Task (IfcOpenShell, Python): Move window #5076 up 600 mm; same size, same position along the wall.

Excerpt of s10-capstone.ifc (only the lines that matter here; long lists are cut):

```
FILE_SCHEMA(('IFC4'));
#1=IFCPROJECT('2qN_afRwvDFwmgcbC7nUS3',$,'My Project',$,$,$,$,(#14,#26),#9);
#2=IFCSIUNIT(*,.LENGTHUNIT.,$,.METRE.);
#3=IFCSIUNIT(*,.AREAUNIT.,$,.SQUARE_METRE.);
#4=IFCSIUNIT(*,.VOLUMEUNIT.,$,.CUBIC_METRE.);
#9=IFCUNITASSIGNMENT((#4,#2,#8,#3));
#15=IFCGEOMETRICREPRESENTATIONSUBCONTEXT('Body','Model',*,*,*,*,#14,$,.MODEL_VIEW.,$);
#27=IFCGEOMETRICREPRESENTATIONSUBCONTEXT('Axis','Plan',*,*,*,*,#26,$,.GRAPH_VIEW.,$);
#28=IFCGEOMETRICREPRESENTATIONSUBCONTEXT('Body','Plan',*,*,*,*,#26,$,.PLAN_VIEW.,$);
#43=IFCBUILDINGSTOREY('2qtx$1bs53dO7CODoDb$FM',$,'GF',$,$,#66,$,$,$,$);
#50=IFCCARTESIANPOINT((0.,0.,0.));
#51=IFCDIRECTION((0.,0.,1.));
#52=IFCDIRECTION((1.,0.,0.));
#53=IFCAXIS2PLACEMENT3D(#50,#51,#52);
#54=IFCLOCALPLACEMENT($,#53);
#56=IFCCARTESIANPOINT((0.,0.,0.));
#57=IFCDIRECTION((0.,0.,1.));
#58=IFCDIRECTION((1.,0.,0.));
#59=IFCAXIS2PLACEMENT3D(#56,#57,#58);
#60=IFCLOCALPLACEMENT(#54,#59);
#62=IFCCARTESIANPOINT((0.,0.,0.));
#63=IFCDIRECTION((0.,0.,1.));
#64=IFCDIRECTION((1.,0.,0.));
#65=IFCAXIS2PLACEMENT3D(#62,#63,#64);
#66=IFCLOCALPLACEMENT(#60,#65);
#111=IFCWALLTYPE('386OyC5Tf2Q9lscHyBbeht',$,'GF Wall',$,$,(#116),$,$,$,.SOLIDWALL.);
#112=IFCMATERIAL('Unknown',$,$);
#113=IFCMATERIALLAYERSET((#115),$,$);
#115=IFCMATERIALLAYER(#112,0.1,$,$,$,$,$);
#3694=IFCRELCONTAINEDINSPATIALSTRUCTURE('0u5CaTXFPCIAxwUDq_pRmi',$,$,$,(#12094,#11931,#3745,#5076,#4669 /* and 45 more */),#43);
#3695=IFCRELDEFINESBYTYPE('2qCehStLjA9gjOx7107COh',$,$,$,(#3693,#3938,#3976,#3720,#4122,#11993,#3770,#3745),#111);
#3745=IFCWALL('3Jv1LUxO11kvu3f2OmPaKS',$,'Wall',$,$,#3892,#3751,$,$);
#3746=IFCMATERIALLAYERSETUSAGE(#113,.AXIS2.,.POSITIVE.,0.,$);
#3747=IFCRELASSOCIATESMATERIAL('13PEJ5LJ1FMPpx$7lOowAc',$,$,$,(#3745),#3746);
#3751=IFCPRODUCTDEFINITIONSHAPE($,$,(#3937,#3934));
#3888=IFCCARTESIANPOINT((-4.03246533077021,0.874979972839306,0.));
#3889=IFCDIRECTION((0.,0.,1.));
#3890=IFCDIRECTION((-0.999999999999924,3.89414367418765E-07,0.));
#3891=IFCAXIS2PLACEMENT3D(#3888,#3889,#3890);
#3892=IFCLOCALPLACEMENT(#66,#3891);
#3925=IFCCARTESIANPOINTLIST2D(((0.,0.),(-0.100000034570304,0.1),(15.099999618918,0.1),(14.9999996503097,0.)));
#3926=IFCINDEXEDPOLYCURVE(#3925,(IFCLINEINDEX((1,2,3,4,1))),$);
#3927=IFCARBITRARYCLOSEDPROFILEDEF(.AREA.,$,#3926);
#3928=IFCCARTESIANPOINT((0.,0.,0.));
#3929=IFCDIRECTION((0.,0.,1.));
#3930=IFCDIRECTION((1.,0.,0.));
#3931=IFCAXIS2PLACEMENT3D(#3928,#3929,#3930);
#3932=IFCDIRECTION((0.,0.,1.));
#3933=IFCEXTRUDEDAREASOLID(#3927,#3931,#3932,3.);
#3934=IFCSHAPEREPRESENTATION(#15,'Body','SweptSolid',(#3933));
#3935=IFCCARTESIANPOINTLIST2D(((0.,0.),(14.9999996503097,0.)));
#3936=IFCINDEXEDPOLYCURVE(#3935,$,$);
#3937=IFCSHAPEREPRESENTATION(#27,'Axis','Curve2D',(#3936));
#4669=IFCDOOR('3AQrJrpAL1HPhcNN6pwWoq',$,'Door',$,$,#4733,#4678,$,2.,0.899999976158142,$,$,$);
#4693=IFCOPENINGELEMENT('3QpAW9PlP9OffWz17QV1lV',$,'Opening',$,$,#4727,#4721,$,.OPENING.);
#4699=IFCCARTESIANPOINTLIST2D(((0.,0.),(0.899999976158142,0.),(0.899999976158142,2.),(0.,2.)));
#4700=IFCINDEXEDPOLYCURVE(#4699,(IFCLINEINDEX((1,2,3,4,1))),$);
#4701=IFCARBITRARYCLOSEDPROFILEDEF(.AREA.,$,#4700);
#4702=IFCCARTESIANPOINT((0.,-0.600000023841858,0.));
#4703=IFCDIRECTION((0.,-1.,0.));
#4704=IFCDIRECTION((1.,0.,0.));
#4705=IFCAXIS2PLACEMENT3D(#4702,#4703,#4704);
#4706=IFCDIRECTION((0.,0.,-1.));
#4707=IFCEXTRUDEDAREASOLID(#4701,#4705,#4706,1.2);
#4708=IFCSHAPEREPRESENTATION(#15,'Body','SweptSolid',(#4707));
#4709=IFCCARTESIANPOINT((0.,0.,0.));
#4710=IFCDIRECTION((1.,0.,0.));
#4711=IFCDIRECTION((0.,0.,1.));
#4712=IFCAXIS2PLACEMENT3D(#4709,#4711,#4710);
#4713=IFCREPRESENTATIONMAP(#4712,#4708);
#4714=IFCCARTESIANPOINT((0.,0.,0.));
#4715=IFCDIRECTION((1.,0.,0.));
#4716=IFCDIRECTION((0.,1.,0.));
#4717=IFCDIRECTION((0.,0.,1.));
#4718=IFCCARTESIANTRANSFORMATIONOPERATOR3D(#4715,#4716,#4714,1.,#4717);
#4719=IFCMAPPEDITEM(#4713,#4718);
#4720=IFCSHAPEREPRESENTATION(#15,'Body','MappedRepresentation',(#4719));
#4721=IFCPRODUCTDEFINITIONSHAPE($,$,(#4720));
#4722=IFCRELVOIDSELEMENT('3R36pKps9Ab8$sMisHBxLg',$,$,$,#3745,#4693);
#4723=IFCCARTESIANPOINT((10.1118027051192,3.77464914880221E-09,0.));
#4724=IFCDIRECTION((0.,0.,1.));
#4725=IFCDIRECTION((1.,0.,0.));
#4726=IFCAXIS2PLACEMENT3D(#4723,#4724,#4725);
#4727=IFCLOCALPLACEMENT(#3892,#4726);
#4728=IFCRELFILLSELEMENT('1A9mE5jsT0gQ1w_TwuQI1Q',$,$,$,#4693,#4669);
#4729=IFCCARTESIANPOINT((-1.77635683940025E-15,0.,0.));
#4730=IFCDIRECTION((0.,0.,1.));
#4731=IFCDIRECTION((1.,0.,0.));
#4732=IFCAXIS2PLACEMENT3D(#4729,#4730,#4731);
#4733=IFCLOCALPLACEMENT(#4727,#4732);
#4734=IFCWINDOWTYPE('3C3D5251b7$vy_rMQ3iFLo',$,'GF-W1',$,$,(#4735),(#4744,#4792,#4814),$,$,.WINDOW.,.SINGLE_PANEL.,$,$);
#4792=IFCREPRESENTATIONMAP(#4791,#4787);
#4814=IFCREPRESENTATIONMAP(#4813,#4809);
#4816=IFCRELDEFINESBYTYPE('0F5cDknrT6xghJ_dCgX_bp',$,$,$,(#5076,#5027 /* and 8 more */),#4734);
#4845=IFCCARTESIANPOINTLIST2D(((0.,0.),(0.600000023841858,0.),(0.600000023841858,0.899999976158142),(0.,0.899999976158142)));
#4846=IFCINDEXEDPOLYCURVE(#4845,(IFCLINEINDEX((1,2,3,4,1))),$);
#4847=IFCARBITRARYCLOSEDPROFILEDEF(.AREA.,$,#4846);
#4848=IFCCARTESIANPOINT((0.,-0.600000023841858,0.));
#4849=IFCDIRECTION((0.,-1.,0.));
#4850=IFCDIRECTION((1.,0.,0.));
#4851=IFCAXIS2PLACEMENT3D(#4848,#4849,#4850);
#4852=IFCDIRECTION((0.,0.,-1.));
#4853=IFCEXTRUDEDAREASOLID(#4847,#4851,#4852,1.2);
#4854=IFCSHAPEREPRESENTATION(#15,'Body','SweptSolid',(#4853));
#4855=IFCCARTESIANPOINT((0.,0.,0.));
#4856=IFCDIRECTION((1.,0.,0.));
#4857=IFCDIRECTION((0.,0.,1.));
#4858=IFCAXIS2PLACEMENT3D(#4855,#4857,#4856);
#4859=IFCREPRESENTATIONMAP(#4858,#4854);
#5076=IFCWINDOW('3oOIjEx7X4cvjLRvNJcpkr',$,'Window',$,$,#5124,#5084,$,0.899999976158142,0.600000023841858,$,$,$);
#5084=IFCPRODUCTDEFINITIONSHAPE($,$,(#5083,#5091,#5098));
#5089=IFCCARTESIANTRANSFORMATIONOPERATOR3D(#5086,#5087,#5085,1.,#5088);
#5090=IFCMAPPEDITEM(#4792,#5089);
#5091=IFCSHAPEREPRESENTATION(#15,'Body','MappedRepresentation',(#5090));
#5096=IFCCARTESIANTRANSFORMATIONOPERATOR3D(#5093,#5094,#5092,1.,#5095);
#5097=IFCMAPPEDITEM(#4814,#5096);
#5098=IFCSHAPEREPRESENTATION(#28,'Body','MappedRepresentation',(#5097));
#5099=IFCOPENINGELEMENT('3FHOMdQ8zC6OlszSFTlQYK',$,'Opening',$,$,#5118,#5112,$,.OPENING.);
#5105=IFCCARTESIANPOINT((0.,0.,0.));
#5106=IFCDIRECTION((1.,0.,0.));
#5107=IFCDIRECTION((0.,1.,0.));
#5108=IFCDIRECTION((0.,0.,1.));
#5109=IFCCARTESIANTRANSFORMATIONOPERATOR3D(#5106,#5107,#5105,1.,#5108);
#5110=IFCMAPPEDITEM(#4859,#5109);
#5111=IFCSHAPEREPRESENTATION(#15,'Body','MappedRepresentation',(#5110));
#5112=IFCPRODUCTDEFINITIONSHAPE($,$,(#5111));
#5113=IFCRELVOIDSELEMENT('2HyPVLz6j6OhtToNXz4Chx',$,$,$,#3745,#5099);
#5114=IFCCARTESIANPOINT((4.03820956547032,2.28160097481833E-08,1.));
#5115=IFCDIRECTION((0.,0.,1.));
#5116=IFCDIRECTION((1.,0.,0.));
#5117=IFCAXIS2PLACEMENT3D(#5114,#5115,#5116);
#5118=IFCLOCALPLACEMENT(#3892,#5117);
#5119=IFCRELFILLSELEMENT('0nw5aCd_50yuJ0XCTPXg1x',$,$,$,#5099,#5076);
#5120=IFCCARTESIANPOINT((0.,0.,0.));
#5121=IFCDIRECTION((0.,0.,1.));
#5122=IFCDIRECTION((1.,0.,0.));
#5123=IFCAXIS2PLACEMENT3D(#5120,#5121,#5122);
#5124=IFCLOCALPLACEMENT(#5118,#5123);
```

```python
import numpy as np
import ifcopenshell
import ifcopenshell.api.geometry
import ifcopenshell.util.placement
import ifcopenshell.util.unit

model = ifcopenshell.open("s10-capstone.ifc")
unit_scale = ifcopenshell.util.unit.calculate_unit_scale(model)

window = model.by_id(5076)
opening = window.FillsVoids[0].RelatingOpeningElement
dz = 0.6 / unit_scale

shift = np.array([0.0, 0.0, dz])
# The window is placed relative to its opening, so it follows when the opening moves.
matrix = ifcopenshell.util.placement.get_local_placement(opening.ObjectPlacement)
matrix[:3, 3] += shift
ifcopenshell.api.geometry.edit_object_placement(
    model, product=opening, matrix=matrix, is_si=False, should_transform_children=True
)

print(f"moved by {dz * unit_scale:+.3f} m")

model.write("s10-capstone_edited.ifc")
```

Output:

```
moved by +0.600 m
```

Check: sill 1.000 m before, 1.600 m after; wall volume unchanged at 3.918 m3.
